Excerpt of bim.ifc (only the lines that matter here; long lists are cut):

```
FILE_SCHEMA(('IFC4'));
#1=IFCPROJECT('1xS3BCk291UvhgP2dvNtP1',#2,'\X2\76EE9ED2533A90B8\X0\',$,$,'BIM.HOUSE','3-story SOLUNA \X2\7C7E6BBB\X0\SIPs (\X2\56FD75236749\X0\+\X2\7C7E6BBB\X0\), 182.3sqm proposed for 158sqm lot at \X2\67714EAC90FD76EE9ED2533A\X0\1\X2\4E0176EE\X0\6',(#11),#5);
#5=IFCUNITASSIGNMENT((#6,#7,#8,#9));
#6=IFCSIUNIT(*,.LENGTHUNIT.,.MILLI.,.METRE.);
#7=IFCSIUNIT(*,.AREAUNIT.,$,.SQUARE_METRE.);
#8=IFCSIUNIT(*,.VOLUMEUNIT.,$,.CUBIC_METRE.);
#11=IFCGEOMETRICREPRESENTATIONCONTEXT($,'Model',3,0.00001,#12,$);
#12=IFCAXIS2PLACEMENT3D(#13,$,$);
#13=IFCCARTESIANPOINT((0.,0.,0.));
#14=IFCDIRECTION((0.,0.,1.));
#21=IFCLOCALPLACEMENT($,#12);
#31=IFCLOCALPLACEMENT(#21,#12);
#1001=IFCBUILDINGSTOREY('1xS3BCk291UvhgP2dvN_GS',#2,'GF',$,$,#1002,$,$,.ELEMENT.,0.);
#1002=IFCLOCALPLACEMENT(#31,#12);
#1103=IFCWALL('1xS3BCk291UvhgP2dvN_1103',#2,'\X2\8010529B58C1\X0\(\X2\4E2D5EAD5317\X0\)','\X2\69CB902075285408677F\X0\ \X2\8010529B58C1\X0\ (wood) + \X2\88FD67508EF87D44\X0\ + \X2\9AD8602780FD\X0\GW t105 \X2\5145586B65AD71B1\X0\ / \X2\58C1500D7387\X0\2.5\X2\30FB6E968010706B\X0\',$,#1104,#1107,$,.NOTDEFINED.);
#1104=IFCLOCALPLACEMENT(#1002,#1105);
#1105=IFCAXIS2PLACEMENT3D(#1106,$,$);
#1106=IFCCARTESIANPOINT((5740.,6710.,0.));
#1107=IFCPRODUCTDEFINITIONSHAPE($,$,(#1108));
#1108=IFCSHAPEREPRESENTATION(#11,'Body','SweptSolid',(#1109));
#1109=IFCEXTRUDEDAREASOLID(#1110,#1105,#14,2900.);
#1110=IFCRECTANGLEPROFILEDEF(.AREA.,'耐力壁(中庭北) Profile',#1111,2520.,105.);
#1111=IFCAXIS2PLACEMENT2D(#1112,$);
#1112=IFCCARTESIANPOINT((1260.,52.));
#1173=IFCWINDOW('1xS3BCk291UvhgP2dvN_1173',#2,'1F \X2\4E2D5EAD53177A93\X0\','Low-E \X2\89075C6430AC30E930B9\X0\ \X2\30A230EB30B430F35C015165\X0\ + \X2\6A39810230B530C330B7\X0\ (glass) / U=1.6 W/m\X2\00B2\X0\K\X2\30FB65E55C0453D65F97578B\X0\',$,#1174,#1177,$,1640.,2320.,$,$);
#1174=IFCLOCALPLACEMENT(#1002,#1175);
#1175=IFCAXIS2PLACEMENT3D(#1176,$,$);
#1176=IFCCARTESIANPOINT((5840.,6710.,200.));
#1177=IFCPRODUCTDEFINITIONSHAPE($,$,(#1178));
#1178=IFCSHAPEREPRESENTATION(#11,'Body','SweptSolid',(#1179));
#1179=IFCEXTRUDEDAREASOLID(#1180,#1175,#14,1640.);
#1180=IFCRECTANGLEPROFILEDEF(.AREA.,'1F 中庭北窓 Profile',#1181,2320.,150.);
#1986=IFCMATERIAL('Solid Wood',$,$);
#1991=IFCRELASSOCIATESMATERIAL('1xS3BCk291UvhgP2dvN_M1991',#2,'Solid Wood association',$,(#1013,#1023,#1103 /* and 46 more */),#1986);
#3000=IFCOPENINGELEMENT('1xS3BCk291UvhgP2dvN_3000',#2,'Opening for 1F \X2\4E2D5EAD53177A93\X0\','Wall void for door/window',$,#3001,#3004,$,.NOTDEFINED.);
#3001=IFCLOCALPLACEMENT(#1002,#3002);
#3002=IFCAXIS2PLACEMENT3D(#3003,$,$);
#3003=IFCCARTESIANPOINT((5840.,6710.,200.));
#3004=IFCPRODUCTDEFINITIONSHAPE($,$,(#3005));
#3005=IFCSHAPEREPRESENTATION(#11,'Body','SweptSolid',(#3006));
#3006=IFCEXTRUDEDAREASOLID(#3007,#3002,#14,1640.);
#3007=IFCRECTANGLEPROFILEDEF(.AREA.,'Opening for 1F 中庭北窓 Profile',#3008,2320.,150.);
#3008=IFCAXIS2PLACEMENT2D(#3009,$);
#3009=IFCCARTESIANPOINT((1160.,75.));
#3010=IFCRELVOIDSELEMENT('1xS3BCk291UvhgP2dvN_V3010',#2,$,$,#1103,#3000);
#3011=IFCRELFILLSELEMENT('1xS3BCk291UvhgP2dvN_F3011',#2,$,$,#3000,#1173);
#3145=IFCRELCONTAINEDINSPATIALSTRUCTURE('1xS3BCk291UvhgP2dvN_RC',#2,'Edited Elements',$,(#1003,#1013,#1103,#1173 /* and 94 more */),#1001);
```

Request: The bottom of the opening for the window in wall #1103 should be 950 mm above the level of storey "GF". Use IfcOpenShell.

```python
import numpy as np
import ifcopenshell
import ifcopenshell.api.geometry
import ifcopenshell.geom
import ifcopenshell.util.element
import ifcopenshell.util.placement
import ifcopenshell.util.shape
import ifcopenshell.util.unit

model = ifcopenshell.open("bim.ifc")
unit_scale = ifcopenshell.util.unit.calculate_unit_scale(model)

window = model.by_id(1173)
opening = window.FillsVoids[0].RelatingOpeningElement
storey = ifcopenshell.util.element.get_container(window, ifc_class="IfcBuildingStorey")
level = ifcopenshell.util.placement.get_local_placement(storey.ObjectPlacement)[2, 3]

# The opening's origin need not be at the sill, so measure its lowest point.
shape = ifcopenshell.geom.create_shape(ifcopenshell.geom.settings(), opening)
bottom = ifcopenshell.util.shape.get_shape_bottom_elevation(shape, shape.geometry) / unit_scale
dz = level + 950.0 - bottom

shift = np.array([0.0, 0.0, dz])
# The window is not placed relative to its opening, so move both.
for product in (opening, window):
    matrix = ifcopenshell.util.placement.get_local_placement(product.ObjectPlacement)
    matrix[:3, 3] += shift
    ifcopenshell.api.geometry.edit_object_placement(model, product=product, matrix=matrix, is_si=False)

print(f"moved by {dz * unit_scale:+.3f} m")

model.write("bim_edited.ifc")
```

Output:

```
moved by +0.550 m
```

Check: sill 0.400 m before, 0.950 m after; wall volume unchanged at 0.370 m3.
